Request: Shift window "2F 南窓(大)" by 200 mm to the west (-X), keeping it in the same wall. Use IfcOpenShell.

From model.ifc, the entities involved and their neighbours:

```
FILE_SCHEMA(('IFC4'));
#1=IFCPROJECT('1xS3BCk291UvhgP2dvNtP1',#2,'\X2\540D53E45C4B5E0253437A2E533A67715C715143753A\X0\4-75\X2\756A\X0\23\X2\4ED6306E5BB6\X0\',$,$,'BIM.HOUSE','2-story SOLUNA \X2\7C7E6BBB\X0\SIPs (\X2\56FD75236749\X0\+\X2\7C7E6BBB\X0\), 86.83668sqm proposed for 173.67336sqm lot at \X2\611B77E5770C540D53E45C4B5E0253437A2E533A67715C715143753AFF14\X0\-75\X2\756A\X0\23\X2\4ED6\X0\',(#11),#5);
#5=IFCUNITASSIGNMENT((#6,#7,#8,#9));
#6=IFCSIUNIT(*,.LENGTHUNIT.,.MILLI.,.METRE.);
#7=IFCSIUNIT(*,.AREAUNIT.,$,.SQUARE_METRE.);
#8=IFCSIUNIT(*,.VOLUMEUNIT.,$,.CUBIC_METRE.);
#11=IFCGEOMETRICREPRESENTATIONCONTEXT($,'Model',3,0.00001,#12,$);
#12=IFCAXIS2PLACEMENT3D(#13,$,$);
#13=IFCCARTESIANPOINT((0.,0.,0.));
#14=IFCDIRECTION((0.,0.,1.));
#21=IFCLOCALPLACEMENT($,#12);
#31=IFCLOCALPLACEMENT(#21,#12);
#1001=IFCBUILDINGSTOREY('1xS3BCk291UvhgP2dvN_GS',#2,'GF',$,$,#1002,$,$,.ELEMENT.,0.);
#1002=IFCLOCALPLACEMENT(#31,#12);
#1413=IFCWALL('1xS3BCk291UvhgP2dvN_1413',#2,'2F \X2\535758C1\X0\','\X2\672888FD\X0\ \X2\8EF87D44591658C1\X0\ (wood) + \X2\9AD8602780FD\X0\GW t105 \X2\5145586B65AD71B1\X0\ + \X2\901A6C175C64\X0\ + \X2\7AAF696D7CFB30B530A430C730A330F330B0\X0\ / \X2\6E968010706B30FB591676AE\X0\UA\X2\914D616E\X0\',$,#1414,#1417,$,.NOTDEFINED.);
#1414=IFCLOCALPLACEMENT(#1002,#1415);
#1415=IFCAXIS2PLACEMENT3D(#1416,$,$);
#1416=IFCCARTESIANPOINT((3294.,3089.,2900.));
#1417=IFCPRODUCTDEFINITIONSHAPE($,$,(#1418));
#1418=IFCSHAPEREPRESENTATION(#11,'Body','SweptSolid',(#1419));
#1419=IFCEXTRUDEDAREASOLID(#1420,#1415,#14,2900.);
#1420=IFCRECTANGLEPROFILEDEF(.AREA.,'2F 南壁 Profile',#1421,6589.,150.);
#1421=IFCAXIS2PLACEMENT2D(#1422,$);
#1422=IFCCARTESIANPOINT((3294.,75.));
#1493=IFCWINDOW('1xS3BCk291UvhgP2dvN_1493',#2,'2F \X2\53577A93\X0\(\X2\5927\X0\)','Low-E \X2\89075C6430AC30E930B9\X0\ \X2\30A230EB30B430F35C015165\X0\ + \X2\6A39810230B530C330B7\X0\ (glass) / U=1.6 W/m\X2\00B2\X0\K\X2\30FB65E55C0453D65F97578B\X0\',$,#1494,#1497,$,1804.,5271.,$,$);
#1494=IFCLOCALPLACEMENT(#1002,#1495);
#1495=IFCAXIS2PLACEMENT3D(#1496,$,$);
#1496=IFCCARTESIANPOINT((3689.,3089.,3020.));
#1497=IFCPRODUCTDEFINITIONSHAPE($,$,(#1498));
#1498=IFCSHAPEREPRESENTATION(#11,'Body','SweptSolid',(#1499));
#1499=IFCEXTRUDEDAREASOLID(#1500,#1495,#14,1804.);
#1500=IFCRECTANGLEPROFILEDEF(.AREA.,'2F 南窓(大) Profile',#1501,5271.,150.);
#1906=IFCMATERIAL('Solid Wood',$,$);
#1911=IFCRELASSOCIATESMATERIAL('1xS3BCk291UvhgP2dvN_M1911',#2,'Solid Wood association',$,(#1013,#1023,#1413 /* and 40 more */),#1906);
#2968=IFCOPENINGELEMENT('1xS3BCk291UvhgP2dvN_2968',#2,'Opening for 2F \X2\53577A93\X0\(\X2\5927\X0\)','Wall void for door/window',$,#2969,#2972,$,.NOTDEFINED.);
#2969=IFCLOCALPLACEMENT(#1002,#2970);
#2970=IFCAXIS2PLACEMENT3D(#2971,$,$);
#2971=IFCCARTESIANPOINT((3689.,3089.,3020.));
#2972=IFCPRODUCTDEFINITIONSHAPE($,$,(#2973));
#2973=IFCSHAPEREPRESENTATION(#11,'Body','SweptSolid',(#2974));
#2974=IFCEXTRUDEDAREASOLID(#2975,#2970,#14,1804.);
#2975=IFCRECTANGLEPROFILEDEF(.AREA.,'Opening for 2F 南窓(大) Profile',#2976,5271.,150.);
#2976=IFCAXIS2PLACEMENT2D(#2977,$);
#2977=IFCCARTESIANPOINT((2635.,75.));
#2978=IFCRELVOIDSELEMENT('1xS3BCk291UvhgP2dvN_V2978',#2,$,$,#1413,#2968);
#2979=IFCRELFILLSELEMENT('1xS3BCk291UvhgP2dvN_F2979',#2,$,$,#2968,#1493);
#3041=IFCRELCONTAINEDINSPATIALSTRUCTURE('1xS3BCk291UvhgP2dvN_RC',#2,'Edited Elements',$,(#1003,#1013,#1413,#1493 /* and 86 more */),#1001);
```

```python
import ifcopenshell
import ifcopenshell.api.geometry
import ifcopenshell.util.placement
import ifcopenshell.util.unit

model = ifcopenshell.open("model.ifc")
unit_scale = ifcopenshell.util.unit.calculate_unit_scale(model)

window = model.by_id(1493)
opening = window.FillsVoids[0].RelatingOpeningElement
wall = opening.VoidsElements[0].RelatingBuildingElement

wall_matrix = ifcopenshell.util.placement.get_local_placement(wall.ObjectPlacement)
shift = wall_matrix[:3, 0] * -0.2 / unit_scale
before = ifcopenshell.util.placement.get_local_placement(window.ObjectPlacement)[:3, 3].copy()

# The window is not placed relative to its opening, so move both.
for product in (opening, window):
    matrix = ifcopenshell.util.placement.get_local_placement(product.ObjectPlacement)
    matrix[:3, 3] += shift
    ifcopenshell.api.geometry.edit_object_placement(model, product=product, matrix=matrix, is_si=False)

after = ifcopenshell.util.placement.get_local_placement(window.ObjectPlacement)[:3, 3]
print("window moved by", (after - before).round(3) + 0.0)

model.write("model-out.ifc")
```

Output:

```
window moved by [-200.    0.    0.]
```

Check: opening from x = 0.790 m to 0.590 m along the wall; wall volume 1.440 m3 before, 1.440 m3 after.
